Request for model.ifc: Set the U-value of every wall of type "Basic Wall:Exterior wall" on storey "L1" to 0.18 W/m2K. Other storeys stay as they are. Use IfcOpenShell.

First a look at what the model holds.

```python
import ifcopenshell
import ifcopenshell.util.element

model = ifcopenshell.open("model.ifc")
print(model.schema)
storey = next(s for s in model.by_type("IfcBuildingStorey") if s.Name == "L1")
walls = [e for e in ifcopenshell.util.element.get_decomposition(storey) if e.is_a("IfcWall")]
seen = {}
for e in walls:
    element_type = ifcopenshell.util.element.get_type(e)
    key = (element_type.Name if element_type != e and element_type else None, ifcopenshell.util.element.get_pset(e, "Pset_WallCommon", "ThermalTransmittance"))
    seen[key] = seen.get(key, 0) + 1
for (name, value), count in sorted(seen.items(), key=str):
    print(count, "x", name, "|", value)
```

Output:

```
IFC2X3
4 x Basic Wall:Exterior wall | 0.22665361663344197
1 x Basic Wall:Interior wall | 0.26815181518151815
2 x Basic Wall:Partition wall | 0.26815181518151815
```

```python
import ifcopenshell
import ifcopenshell.api.pset
import ifcopenshell.util.element

model = ifcopenshell.open("model.ifc")

storey = next(s for s in model.by_type("IfcBuildingStorey") if s.Name == "L1")
walls = [e for e in ifcopenshell.util.element.get_decomposition(storey) if e.is_a("IfcWall")]

count = 0
for e in walls:
    element_type = ifcopenshell.util.element.get_type(e)
    if element_type in (None, e) or element_type.Name != "Basic Wall:Exterior wall":
        continue
    # add_pset returns the element's existing set when there is one.
    pset = ifcopenshell.api.pset.add_pset(model, product=e, name="Pset_WallCommon")
    ifcopenshell.api.pset.edit_pset(model, pset=pset, properties={"ThermalTransmittance": 0.18})
    count += 1

print(count, "walls updated")

model.write("model_edited.ifc")
```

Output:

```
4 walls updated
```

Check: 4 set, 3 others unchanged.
